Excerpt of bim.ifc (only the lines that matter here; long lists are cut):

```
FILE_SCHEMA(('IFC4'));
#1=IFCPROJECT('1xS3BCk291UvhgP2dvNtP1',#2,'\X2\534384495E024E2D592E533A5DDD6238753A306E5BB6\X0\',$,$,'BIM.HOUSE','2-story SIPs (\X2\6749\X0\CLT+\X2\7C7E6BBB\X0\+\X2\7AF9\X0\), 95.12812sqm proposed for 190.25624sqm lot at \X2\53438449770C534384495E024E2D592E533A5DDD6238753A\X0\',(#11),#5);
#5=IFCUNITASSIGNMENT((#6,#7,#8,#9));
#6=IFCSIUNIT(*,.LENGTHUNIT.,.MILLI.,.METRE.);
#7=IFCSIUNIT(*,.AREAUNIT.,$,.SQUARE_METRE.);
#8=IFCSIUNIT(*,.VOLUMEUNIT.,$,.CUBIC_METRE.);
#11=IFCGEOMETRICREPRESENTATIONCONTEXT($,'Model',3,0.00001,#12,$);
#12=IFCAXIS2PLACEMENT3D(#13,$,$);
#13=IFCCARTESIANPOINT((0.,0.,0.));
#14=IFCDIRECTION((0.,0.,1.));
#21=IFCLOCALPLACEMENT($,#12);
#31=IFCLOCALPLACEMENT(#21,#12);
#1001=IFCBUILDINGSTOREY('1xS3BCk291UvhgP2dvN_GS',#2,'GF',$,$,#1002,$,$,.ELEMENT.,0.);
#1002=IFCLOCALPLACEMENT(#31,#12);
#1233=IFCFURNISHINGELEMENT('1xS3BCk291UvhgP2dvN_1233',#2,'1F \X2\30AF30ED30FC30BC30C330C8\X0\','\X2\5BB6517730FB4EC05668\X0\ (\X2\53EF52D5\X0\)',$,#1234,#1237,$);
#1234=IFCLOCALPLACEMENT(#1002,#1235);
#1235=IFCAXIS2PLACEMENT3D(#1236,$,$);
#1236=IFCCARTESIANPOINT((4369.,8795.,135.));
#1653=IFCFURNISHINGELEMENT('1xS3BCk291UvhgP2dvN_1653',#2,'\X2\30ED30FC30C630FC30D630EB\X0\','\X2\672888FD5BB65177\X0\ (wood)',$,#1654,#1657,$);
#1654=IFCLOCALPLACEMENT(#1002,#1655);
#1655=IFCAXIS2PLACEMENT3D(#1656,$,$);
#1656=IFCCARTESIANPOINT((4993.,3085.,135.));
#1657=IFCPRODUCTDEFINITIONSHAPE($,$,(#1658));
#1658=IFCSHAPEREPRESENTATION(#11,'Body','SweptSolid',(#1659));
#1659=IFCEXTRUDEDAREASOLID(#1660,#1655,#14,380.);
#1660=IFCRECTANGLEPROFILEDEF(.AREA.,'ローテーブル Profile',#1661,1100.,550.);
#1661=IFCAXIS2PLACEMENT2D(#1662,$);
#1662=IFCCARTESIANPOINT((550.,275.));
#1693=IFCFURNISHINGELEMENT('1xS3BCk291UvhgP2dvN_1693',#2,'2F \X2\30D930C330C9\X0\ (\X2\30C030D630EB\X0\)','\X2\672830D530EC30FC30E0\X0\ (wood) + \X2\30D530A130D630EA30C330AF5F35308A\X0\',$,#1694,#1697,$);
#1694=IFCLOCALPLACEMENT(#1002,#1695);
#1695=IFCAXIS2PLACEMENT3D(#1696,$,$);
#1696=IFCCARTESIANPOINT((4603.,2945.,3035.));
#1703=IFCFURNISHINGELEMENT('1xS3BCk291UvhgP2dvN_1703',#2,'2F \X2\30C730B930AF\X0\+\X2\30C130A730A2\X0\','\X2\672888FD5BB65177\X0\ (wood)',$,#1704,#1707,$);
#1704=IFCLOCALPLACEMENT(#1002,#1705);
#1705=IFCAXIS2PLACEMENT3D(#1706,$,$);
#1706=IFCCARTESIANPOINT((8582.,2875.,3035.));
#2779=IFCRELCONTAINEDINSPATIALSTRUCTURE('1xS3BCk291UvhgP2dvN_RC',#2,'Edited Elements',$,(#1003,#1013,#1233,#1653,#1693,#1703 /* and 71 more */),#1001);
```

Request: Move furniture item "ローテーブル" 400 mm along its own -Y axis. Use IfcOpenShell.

```python
import ifcopenshell
import ifcopenshell.api.geometry
import ifcopenshell.util.placement
import ifcopenshell.util.unit

model = ifcopenshell.open("bim.ifc")
unit_scale = ifcopenshell.util.unit.calculate_unit_scale(model)

item = model.by_guid("1xS3BCk291UvhgP2dvN_1653")
matrix = ifcopenshell.util.placement.get_local_placement(item.ObjectPlacement)
matrix[:3, 3] -= matrix[:3, 1] * 0.4 / unit_scale
ifcopenshell.api.geometry.edit_object_placement(model, product=item, matrix=matrix, is_si=False)

print(ifcopenshell.util.placement.get_local_placement(item.ObjectPlacement).round(3) + 0.0)

model.write("bim_v2.ifc")
```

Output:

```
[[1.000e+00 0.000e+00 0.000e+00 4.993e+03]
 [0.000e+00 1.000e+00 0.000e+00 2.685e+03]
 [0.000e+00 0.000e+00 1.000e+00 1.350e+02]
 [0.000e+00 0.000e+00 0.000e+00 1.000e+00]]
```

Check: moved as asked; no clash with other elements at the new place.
